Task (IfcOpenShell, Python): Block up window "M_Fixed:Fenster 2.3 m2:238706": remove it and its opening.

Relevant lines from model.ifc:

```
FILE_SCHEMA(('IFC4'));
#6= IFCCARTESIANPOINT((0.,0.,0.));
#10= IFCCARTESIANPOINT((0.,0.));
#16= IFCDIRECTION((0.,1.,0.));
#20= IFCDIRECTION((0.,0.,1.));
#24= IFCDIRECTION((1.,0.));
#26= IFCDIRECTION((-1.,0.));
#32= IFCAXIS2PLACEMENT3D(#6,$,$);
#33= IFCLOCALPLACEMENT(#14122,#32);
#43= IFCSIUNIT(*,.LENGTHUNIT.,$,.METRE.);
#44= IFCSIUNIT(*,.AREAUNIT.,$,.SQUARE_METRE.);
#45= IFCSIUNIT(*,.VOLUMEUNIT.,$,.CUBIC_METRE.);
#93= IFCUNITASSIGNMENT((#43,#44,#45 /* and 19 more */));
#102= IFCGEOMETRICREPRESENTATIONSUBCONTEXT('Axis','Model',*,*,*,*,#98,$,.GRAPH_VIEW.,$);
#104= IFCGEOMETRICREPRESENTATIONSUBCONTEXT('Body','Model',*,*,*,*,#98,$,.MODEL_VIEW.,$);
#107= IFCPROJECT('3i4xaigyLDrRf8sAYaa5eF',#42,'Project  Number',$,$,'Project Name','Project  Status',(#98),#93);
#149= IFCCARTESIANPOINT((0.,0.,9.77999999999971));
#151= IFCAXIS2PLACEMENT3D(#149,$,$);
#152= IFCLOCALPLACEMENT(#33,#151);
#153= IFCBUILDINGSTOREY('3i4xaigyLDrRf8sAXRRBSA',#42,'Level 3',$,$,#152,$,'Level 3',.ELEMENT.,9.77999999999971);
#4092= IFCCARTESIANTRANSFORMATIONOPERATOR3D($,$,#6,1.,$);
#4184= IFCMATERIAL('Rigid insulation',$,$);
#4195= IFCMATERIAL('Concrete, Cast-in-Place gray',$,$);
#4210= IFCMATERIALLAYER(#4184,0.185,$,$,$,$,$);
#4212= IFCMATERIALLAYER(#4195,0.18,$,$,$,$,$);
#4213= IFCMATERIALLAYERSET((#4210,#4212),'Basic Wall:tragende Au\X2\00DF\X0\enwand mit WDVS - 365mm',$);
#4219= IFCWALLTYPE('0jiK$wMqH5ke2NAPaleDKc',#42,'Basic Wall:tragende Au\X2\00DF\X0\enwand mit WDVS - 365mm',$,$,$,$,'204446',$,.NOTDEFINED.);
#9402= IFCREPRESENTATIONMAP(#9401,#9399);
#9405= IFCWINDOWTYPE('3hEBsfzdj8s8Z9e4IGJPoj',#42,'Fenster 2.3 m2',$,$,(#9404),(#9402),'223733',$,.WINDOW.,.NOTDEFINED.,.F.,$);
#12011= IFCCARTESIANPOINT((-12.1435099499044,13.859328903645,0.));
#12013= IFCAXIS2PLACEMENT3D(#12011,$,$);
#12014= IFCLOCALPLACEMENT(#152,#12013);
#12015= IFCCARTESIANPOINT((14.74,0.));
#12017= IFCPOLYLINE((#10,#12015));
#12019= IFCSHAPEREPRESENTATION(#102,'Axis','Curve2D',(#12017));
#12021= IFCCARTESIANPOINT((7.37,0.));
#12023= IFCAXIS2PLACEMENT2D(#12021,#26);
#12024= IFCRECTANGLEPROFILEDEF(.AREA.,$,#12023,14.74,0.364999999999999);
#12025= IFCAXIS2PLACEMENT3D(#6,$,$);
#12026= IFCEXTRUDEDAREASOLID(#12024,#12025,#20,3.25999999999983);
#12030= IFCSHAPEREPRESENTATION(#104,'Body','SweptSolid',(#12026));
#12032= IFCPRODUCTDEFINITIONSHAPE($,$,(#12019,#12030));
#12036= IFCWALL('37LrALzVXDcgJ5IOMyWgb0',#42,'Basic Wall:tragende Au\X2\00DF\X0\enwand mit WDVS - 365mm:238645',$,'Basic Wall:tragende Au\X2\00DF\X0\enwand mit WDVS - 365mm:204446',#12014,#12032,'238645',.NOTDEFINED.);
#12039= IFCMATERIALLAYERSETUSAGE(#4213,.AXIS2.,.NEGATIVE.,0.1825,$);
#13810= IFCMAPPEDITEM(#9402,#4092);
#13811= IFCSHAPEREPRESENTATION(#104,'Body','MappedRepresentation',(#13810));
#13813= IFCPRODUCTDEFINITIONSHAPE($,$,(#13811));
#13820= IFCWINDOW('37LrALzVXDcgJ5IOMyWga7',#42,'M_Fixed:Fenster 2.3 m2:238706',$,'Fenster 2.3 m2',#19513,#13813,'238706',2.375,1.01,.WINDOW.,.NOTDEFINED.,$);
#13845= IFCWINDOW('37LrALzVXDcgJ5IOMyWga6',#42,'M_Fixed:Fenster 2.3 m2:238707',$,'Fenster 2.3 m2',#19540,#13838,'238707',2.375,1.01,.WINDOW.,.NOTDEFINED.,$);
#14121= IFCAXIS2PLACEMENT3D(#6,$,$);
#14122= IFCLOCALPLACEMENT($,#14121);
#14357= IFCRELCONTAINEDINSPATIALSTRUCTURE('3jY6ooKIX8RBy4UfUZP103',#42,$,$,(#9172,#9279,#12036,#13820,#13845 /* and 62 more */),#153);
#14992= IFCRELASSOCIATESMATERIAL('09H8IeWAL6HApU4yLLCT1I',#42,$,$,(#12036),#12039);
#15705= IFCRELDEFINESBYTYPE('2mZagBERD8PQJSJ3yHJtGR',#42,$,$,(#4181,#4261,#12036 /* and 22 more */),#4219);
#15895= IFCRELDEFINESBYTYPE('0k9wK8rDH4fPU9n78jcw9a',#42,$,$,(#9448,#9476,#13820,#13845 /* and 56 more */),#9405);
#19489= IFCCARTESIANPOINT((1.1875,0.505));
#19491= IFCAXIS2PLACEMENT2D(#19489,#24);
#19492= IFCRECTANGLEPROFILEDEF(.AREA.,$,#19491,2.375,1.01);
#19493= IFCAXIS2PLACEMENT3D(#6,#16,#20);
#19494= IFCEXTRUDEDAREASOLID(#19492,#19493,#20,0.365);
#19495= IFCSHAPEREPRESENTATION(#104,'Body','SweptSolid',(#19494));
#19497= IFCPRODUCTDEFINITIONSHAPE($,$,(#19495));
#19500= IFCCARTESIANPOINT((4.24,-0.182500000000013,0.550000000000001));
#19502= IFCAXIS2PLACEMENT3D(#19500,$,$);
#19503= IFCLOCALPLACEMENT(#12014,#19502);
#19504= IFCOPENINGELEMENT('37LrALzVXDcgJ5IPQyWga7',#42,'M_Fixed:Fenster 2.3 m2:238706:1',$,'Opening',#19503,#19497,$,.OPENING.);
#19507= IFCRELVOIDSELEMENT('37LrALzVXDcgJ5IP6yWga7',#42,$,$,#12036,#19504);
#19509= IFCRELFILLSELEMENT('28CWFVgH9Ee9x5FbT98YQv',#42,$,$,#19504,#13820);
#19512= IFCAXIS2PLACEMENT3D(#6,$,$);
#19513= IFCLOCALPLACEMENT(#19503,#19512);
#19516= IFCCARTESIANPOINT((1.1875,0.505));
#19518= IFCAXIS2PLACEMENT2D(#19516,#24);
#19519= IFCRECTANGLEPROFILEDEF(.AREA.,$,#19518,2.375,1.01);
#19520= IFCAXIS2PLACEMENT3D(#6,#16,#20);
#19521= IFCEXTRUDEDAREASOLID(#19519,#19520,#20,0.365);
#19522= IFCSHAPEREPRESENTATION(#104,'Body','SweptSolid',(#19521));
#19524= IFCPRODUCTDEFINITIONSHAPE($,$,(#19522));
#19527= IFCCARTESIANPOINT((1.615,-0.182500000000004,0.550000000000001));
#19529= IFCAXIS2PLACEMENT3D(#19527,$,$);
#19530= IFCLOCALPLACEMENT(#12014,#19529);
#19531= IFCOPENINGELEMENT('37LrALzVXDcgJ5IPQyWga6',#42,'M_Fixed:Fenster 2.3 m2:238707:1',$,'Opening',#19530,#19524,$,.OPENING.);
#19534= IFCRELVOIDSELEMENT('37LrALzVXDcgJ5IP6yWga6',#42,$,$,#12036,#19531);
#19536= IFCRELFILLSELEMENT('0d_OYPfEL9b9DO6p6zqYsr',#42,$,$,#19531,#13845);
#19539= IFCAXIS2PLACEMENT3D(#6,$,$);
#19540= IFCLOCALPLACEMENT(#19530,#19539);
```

```python
import ifcopenshell
import ifcopenshell.api.feature
import ifcopenshell.api.root
import ifcopenshell.geom
import ifcopenshell.util.shape

model = ifcopenshell.open("model.ifc")
settings = ifcopenshell.geom.settings()


def volume(element):
    """Net volume in cubic metres, openings subtracted."""
    shape = ifcopenshell.geom.create_shape(settings, element)
    return ifcopenshell.util.shape.get_volume(shape.geometry)


window = model.by_id(13820)
opening = window.FillsVoids[0].RelatingOpeningElement
wall = opening.VoidsElements[0].RelatingBuildingElement
before = volume(wall)

ifcopenshell.api.root.remove_product(model, product=window)
ifcopenshell.api.feature.remove_feature(model, feature=opening)

after = volume(wall)

print(f"wall volume {before:.3f} -> {after:.3f} m3")

model.write("model_updated.ifc")
```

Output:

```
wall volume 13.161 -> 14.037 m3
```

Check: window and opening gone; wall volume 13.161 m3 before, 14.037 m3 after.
